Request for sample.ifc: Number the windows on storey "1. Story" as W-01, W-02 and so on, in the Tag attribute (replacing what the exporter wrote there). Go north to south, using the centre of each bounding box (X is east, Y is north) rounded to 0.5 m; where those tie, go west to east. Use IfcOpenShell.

First a look at what the model holds.

```python
import ifcopenshell
import ifcopenshell.util.element
import ifcopenshell.util.placement

model = ifcopenshell.open("sample.ifc")
print(model.schema)
storey = next(s for s in model.by_type("IfcBuildingStorey") if s.Name == "1. Story")
windows = [e for e in ifcopenshell.util.element.get_decomposition(storey) if e.is_a("IfcWindow")]
for e in sorted(windows, key=lambda e: e.id()):
    origin = ifcopenshell.util.placement.get_local_placement(e.ObjectPlacement)[:3, 3]
    print(e.id(), e.Tag, e.Name, origin.round(2) + 0.0, sep=" | ")
```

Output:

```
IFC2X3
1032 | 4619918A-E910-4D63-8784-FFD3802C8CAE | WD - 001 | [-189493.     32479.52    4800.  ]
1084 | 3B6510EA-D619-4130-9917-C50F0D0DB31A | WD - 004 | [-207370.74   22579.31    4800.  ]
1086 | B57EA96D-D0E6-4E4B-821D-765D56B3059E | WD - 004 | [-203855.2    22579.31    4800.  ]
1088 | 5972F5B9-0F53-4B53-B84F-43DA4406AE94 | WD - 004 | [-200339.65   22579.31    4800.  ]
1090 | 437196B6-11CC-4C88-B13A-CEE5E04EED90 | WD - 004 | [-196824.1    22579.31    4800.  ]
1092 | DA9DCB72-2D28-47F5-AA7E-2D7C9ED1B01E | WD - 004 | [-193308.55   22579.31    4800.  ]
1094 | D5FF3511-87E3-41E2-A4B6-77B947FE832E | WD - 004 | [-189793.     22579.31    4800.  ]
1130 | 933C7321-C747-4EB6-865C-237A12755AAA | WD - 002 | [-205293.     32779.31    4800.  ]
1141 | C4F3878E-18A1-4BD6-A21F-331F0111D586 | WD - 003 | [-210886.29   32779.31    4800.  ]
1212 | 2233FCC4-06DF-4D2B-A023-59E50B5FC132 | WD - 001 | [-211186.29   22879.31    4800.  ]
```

```python
import ifcopenshell
import ifcopenshell.geom
import ifcopenshell.util.element
import ifcopenshell.util.shape

model = ifcopenshell.open("sample.ifc")
settings = ifcopenshell.geom.settings()
settings.set("use-world-coords", True)


def centre(element):
    shape = ifcopenshell.geom.create_shape(settings, element)
    return ifcopenshell.util.shape.get_bbox_centroid(shape.geometry)


storey = next(s for s in model.by_type("IfcBuildingStorey") if s.Name == "1. Story")
windows = [e for e in ifcopenshell.util.element.get_decomposition(storey) if e.is_a("IfcWindow")]

# Insertion points can sit at a corner or the storey origin, so sort by the geometry (in metres).
centres = {e: centre(e) for e in windows}
windows.sort(key=lambda e: (-round(centres[e][1] / 0.5), centres[e][0]))

for i, e in enumerate(windows, start=1):
    number = f"W-{i:02d}"
    e.Tag = number
    print(e.id(), number)

model.write("sample_updated.ifc")
```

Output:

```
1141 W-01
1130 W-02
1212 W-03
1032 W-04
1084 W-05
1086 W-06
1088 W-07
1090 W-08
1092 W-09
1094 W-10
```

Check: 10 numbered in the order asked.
